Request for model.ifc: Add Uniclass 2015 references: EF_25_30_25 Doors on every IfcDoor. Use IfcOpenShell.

First a look at what the model holds.

```python
import ifcopenshell

model = ifcopenshell.open("model.ifc")
print(model.schema)
print("classifications:", [c.Name for c in model.by_type("IfcClassification")])
for ifc_class in ("IfcDoor", "IfcRoof", "IfcStair", "IfcWall", "IfcWindow"):
    print(ifc_class, len(model.by_type(ifc_class)))
```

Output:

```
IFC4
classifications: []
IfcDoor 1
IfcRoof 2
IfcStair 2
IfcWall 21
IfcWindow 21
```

```python
import ifcopenshell
import ifcopenshell.api.classification

model = ifcopenshell.open("model.ifc")

system = ifcopenshell.api.classification.add_classification(model, classification="Uniclass 2015")

codes = {
    "IfcDoor": ("EF_25_30_25", "Doors"),
}
for ifc_class, (code, name) in codes.items():
    products = model.by_type(ifc_class)
    ifcopenshell.api.classification.add_reference(
        model, products=products, classification=system, identification=code, name=name
    )
    print(code, len(products))

model.write("model_rev.ifc")
```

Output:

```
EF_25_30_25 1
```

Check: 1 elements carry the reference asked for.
